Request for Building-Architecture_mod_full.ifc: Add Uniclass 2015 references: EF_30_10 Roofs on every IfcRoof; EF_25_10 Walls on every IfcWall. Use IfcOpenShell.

First a look at what the model holds.

```python
import ifcopenshell

model = ifcopenshell.open("Building-Architecture_mod_full.ifc")
print(model.schema)
print("classifications:", [c.Name for c in model.by_type("IfcClassification")])
for ifc_class in ("IfcDoor", "IfcRoof", "IfcStair", "IfcWall", "IfcWindow"):
    print(ifc_class, len(model.by_type(ifc_class)))
```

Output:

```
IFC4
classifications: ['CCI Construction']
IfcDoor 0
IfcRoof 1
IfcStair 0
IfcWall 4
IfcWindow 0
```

```python
import ifcopenshell
import ifcopenshell.api.classification

model = ifcopenshell.open("Building-Architecture_mod_full.ifc")

system = ifcopenshell.api.classification.add_classification(model, classification="Uniclass 2015")

codes = {
    "IfcRoof": ("EF_30_10", "Roofs"),
    "IfcWall": ("EF_25_10", "Walls"),
}
for ifc_class, (code, name) in codes.items():
    products = model.by_type(ifc_class)
    ifcopenshell.api.classification.add_reference(
        model, products=products, classification=system, identification=code, name=name
    )
    print(code, len(products))

model.write("Building-Architecture_mod_full_rev.ifc")
```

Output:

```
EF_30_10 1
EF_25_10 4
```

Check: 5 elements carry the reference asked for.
